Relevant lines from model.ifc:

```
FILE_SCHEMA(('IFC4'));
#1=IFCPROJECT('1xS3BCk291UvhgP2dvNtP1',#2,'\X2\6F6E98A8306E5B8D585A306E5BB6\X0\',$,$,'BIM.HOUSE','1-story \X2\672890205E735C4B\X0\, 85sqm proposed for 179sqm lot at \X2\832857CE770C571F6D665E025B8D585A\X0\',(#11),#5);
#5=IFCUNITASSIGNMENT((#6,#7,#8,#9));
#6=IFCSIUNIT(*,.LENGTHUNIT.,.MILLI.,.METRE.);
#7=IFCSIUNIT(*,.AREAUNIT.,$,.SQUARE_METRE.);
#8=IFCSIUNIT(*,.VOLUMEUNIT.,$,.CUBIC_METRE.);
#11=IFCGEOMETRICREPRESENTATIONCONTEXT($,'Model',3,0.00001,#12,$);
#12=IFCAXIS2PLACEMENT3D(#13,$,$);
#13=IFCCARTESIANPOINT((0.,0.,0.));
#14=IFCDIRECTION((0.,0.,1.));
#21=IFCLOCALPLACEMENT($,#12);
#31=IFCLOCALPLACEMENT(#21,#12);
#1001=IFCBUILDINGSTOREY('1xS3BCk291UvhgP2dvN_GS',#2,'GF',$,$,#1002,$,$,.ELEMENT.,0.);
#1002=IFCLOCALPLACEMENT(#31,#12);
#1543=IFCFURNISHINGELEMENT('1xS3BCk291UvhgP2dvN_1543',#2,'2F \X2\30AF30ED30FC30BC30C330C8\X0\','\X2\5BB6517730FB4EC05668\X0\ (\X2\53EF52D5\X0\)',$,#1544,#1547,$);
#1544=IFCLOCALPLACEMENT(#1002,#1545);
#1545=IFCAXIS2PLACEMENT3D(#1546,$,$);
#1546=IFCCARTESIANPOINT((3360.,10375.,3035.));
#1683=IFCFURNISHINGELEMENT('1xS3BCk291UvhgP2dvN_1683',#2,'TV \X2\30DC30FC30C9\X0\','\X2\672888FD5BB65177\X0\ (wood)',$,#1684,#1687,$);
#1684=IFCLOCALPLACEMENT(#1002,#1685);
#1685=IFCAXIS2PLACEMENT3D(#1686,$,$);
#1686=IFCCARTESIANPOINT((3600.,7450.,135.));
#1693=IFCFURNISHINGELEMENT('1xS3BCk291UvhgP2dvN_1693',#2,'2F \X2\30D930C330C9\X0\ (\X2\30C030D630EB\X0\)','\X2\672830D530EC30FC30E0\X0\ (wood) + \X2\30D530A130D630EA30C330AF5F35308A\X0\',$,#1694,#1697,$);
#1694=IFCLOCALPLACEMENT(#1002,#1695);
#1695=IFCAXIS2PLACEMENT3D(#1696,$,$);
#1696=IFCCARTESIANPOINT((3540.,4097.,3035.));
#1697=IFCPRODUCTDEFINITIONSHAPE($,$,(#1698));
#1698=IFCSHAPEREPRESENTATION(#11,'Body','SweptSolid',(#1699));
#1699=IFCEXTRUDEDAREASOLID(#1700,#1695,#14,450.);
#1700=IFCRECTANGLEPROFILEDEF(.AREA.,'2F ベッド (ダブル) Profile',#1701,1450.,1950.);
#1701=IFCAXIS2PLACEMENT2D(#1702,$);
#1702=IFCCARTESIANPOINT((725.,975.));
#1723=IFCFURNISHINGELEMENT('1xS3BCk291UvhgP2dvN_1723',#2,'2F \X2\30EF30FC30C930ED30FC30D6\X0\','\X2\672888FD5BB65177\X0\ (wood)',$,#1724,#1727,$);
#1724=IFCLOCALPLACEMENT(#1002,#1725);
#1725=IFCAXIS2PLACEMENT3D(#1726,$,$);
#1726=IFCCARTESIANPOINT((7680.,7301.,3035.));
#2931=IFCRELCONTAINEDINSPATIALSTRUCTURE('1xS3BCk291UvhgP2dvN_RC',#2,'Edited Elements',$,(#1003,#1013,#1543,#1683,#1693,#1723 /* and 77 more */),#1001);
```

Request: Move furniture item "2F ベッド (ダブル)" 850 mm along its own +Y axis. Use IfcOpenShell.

```python
import ifcopenshell
import ifcopenshell.api.geometry
import ifcopenshell.util.placement
import ifcopenshell.util.unit

model = ifcopenshell.open("model.ifc")
unit_scale = ifcopenshell.util.unit.calculate_unit_scale(model)

item = model.by_guid("1xS3BCk291UvhgP2dvN_1693")
matrix = ifcopenshell.util.placement.get_local_placement(item.ObjectPlacement)
matrix[:3, 3] += matrix[:3, 1] * 0.85 / unit_scale
ifcopenshell.api.geometry.edit_object_placement(model, product=item, matrix=matrix, is_si=False)

print(ifcopenshell.util.placement.get_local_placement(item.ObjectPlacement).round(3) + 0.0)

model.write("model_updated.ifc")
```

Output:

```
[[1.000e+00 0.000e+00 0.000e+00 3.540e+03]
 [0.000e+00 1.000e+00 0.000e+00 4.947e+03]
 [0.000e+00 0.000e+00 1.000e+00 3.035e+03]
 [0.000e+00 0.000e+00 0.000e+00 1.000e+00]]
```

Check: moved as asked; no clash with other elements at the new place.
